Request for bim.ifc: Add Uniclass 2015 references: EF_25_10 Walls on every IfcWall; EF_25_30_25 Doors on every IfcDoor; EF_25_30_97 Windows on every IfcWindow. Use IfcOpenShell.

First a look at what the model holds.

```python
import ifcopenshell

model = ifcopenshell.open("bim.ifc")
print(model.schema)
print("classifications:", [c.Name for c in model.by_type("IfcClassification")])
for ifc_class in ("IfcDoor", "IfcRoof", "IfcStair", "IfcWall", "IfcWindow"):
    print(ifc_class, len(model.by_type(ifc_class)))
```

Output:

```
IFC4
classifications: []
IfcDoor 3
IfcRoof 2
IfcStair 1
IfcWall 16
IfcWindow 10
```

```python
import ifcopenshell
import ifcopenshell.api.classification

model = ifcopenshell.open("bim.ifc")

system = ifcopenshell.api.classification.add_classification(model, classification="Uniclass 2015")

codes = {
    "IfcWall": ("EF_25_10", "Walls"),
    "IfcDoor": ("EF_25_30_25", "Doors"),
    "IfcWindow": ("EF_25_30_97", "Windows"),
}
for ifc_class, (code, name) in codes.items():
    products = model.by_type(ifc_class)
    ifcopenshell.api.classification.add_reference(
        model, products=products, classification=system, identification=code, name=name
    )
    print(code, len(products))

model.write("bim_rev.ifc")
```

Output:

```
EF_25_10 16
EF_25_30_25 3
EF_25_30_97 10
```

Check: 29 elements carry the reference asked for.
